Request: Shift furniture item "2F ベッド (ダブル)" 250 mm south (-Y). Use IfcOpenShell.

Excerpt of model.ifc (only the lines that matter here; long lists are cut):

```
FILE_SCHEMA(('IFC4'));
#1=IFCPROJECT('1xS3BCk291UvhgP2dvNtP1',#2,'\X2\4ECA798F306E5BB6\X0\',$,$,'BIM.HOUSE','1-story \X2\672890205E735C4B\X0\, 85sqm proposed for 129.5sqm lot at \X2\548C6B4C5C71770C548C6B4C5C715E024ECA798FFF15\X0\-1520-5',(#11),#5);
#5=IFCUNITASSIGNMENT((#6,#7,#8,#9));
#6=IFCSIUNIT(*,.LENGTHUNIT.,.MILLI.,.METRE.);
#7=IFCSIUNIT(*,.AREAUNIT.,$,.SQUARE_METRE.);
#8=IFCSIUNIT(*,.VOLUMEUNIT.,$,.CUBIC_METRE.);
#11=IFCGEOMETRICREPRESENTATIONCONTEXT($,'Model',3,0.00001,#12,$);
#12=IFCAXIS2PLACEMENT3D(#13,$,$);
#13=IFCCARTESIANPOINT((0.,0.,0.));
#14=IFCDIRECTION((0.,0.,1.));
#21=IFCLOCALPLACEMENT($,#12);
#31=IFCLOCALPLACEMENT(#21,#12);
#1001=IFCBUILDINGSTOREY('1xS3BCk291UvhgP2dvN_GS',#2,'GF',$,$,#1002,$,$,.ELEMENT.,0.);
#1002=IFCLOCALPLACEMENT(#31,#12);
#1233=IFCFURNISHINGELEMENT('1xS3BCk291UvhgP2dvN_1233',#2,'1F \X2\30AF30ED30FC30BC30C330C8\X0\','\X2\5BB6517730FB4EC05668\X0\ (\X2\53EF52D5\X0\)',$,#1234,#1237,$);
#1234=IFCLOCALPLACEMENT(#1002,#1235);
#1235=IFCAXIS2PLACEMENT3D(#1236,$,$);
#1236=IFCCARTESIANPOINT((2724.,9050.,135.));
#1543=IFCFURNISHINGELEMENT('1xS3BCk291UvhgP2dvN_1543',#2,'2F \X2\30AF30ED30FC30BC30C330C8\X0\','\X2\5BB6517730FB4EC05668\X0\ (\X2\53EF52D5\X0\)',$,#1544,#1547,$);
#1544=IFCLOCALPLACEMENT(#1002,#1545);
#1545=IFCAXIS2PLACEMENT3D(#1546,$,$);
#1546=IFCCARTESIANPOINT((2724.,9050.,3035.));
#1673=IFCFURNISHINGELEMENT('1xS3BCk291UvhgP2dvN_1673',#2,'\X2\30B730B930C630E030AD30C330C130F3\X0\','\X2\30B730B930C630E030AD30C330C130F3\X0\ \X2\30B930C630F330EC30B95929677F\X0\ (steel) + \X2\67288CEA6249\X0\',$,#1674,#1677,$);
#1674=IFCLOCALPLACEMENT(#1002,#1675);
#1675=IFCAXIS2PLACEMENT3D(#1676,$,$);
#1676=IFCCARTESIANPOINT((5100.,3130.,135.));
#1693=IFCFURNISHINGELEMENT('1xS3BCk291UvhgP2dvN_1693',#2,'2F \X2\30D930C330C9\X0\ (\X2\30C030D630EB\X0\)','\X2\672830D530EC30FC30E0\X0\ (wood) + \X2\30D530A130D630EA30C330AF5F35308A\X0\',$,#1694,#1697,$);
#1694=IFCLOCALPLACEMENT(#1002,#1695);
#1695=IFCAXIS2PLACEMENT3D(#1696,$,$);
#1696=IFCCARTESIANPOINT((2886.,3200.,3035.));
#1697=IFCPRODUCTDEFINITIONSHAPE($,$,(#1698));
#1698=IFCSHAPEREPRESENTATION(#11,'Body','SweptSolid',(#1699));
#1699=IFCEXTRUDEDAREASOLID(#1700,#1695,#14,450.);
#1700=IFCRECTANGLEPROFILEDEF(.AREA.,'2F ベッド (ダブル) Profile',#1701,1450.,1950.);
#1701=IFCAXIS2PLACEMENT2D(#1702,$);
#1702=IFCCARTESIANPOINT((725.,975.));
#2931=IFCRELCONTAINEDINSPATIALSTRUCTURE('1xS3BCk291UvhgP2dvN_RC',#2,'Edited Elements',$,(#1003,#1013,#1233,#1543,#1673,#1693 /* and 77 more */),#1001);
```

```python
import ifcopenshell
import ifcopenshell.api.geometry
import ifcopenshell.util.placement

model = ifcopenshell.open("model.ifc")

item = model.by_guid("1xS3BCk291UvhgP2dvN_1693")
matrix = ifcopenshell.util.placement.get_local_placement(item.ObjectPlacement)
matrix[1, 3] -= 250.0
ifcopenshell.api.geometry.edit_object_placement(model, product=item, matrix=matrix, is_si=False)

print(ifcopenshell.util.placement.get_local_placement(item.ObjectPlacement).round(3) + 0.0)

model.write("model_rev.ifc")
```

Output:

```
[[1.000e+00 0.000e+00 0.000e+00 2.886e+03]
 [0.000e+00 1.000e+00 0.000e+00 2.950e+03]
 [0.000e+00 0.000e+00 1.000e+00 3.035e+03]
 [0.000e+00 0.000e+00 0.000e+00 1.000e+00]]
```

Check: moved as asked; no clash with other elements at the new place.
